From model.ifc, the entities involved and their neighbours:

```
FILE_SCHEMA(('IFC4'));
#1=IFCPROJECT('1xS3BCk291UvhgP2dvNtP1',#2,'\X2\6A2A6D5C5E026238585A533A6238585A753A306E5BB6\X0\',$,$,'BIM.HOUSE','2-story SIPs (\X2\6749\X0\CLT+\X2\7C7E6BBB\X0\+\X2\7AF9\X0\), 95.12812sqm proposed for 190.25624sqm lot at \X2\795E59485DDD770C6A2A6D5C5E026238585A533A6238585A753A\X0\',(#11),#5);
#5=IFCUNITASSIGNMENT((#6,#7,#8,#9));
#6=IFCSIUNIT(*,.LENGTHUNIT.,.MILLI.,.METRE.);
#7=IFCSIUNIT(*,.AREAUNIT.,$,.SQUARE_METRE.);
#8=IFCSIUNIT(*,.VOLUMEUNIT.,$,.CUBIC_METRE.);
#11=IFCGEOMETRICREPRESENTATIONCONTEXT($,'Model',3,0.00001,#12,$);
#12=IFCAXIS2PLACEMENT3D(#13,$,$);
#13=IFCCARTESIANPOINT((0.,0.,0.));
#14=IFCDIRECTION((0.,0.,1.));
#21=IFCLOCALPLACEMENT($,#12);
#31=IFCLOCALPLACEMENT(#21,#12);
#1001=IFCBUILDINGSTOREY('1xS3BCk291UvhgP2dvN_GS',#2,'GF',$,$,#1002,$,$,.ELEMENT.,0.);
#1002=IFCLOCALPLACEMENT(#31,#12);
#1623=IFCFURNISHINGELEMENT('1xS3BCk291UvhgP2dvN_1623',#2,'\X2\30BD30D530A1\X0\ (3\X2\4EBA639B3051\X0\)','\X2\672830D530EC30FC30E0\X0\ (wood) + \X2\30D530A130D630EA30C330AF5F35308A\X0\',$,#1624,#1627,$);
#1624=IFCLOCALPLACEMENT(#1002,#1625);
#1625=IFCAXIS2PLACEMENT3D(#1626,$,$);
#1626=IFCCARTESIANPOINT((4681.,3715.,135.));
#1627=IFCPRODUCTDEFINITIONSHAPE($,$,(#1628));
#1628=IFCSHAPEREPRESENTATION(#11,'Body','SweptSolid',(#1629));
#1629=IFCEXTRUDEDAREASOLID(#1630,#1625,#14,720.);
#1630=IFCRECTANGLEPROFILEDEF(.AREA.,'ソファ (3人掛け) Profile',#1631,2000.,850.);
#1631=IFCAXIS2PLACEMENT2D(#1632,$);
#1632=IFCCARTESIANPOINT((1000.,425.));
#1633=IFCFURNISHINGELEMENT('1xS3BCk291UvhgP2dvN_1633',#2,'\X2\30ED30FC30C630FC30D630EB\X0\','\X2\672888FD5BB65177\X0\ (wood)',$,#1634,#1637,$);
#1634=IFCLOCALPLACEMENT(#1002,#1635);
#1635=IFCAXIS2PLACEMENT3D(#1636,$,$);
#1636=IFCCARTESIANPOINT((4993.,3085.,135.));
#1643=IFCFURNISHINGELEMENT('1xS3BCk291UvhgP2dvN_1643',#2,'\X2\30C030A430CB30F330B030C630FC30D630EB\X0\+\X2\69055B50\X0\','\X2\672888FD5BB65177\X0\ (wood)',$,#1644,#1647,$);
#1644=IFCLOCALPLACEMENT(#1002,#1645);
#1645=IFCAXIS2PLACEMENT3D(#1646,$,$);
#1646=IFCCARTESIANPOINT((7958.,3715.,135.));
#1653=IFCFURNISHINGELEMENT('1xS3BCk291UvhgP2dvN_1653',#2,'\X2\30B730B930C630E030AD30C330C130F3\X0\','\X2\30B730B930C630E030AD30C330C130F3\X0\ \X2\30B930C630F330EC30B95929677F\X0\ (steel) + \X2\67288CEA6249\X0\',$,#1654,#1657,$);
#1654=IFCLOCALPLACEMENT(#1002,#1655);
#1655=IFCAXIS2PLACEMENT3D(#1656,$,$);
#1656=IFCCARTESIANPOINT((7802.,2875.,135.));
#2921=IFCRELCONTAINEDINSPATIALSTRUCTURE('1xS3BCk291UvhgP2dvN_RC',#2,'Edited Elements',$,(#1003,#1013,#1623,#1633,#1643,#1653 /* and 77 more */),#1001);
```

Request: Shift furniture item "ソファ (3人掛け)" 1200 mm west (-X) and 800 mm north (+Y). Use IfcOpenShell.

```python
import ifcopenshell
import ifcopenshell.api.geometry
import ifcopenshell.util.placement
import ifcopenshell.util.unit

model = ifcopenshell.open("model.ifc")
unit_scale = ifcopenshell.util.unit.calculate_unit_scale(model)

item = model.by_id(1623)
matrix = ifcopenshell.util.placement.get_local_placement(item.ObjectPlacement)
matrix[0, 3] -= 1.2 / unit_scale
matrix[1, 3] += 0.8 / unit_scale
ifcopenshell.api.geometry.edit_object_placement(model, product=item, matrix=matrix, is_si=False)

print(ifcopenshell.util.placement.get_local_placement(item.ObjectPlacement).round(3) + 0.0)

model.write("model_updated.ifc")
```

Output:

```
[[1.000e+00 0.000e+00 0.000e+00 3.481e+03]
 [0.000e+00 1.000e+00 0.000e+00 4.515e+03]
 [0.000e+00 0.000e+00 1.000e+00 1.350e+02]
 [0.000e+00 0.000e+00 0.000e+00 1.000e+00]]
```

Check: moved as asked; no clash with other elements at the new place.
